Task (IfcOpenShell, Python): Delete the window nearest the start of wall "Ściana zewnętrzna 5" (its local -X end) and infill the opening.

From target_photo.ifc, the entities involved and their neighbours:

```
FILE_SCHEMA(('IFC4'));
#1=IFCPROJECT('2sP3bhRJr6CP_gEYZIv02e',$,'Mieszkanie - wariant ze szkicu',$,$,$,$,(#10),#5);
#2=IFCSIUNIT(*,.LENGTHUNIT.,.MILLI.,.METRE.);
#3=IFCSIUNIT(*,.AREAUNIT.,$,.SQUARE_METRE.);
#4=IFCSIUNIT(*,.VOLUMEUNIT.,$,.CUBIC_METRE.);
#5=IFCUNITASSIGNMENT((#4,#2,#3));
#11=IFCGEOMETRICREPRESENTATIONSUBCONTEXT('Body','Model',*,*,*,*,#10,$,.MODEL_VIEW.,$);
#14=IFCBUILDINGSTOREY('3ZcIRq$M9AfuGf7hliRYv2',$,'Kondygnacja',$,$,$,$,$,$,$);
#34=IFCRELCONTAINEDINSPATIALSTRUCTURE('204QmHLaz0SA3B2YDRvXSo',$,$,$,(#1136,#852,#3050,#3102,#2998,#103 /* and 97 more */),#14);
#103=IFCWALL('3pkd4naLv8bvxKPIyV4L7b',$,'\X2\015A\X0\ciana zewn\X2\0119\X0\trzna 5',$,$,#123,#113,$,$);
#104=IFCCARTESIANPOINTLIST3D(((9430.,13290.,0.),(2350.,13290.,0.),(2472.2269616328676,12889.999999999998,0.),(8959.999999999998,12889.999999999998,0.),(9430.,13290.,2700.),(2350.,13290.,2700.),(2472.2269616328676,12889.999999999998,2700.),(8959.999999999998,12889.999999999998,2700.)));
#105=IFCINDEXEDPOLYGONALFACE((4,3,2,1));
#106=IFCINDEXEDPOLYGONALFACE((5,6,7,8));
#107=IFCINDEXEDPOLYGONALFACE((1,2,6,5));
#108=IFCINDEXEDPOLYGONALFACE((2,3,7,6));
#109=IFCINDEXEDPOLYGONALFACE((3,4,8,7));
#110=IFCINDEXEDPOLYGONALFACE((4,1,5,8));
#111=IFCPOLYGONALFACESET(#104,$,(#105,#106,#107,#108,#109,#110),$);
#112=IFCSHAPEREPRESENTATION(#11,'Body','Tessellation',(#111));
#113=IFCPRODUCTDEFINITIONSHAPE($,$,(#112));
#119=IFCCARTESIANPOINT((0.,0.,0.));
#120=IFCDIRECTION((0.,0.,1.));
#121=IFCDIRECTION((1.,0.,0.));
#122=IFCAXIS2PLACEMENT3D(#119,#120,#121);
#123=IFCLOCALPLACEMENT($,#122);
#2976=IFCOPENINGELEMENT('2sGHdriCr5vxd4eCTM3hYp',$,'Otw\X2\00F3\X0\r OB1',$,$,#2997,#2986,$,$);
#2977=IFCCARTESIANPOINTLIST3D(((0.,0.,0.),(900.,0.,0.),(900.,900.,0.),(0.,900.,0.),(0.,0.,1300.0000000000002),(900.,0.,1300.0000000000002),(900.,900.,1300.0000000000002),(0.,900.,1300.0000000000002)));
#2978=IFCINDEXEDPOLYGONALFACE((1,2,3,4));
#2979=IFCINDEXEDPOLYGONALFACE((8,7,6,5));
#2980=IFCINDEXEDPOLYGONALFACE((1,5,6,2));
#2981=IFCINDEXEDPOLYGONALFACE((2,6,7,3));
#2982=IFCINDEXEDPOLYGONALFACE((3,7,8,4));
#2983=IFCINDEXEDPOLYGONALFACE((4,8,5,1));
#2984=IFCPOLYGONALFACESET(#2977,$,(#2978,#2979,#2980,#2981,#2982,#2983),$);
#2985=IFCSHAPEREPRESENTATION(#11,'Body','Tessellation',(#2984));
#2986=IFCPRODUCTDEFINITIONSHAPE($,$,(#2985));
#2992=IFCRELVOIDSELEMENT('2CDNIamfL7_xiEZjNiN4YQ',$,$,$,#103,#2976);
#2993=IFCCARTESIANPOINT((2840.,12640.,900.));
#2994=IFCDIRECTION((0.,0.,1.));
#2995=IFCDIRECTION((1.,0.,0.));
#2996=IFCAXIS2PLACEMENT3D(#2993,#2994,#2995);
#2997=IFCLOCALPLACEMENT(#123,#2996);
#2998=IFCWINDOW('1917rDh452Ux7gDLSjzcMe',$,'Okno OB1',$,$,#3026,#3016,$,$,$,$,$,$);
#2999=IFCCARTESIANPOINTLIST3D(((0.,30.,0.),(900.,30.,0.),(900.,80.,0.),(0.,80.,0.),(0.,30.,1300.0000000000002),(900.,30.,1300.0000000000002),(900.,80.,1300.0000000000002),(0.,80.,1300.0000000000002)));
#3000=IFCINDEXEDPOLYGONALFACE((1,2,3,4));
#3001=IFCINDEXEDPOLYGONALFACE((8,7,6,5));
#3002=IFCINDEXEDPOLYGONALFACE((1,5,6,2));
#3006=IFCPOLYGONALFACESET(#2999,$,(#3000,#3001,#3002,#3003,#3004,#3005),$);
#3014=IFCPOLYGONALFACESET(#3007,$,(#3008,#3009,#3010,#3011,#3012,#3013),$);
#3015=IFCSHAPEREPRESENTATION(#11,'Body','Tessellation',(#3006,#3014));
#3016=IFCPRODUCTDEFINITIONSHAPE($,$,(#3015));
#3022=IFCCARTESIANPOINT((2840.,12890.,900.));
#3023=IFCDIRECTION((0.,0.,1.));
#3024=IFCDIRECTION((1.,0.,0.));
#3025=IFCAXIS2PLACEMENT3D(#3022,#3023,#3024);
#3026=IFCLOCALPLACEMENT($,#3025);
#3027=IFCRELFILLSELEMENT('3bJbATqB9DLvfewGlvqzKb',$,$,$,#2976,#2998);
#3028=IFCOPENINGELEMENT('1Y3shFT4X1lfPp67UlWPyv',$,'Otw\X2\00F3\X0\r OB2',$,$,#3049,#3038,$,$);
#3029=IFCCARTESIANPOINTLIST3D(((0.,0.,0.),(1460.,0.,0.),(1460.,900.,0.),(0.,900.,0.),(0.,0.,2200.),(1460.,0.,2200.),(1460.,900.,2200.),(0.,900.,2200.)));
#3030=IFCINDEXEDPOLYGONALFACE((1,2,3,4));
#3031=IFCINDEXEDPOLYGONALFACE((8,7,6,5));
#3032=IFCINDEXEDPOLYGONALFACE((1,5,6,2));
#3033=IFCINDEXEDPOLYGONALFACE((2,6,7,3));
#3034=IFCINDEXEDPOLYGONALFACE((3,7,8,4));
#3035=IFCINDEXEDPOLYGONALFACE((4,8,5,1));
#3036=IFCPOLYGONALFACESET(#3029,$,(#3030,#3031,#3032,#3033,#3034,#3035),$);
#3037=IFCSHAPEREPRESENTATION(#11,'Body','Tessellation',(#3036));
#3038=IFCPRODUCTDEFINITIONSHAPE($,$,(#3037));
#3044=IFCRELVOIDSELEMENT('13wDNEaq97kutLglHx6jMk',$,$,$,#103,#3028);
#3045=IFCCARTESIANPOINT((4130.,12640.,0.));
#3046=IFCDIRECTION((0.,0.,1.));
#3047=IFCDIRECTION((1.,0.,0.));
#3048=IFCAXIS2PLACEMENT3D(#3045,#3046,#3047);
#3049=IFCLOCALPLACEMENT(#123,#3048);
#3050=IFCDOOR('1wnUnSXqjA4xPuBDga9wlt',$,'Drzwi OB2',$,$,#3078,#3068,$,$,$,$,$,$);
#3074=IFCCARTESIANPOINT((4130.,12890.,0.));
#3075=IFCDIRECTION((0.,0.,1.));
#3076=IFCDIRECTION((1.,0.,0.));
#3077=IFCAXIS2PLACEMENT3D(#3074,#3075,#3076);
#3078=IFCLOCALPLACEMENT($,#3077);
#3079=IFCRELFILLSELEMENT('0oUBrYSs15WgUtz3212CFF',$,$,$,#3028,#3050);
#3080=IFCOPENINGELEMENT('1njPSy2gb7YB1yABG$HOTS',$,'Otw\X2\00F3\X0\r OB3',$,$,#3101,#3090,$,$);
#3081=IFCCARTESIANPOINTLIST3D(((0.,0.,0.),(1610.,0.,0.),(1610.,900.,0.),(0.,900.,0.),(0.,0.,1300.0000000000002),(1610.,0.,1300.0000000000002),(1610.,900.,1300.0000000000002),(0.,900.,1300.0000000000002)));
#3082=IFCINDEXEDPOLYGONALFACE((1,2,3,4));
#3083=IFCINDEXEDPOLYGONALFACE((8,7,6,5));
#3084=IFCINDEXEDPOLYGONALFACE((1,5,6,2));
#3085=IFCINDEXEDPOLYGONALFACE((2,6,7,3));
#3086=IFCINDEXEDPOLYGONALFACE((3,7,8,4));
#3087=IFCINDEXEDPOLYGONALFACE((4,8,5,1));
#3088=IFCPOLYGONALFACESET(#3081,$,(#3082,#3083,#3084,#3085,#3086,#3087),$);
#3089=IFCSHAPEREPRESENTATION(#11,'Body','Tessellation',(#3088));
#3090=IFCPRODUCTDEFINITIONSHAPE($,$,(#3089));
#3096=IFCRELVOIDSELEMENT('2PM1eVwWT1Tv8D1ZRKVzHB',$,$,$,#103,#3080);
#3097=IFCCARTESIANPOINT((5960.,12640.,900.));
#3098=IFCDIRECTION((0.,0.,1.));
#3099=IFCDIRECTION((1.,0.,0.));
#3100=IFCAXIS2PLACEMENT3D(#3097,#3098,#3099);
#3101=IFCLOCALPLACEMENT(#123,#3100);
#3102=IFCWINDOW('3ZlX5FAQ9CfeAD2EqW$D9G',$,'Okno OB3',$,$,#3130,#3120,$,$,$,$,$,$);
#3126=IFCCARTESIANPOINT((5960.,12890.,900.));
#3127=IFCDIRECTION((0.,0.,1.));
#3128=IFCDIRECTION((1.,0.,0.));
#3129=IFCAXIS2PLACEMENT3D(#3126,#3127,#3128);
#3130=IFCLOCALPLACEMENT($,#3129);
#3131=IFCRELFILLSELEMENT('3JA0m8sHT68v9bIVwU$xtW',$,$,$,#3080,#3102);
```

```python
import ifcopenshell
import ifcopenshell.api.feature
import ifcopenshell.api.root
import ifcopenshell.geom
import ifcopenshell.util.shape

model = ifcopenshell.open("target_photo.ifc")
settings = ifcopenshell.geom.settings()


def volume(element):
    """Net volume in cubic metres, openings subtracted."""
    shape = ifcopenshell.geom.create_shape(settings, element)
    return ifcopenshell.util.shape.get_volume(shape.geometry)


window = model.by_guid("1917rDh452Ux7gDLSjzcMe")
opening = window.FillsVoids[0].RelatingOpeningElement
wall = opening.VoidsElements[0].RelatingBuildingElement
before = volume(wall)

ifcopenshell.api.root.remove_product(model, product=window)
ifcopenshell.api.feature.remove_feature(model, feature=opening)

after = volume(wall)

print(f"wall volume {before:.3f} -> {after:.3f} m3")

model.write("target_photo_updated.ifc")
```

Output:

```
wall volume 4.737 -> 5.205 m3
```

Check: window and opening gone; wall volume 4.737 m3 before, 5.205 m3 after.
